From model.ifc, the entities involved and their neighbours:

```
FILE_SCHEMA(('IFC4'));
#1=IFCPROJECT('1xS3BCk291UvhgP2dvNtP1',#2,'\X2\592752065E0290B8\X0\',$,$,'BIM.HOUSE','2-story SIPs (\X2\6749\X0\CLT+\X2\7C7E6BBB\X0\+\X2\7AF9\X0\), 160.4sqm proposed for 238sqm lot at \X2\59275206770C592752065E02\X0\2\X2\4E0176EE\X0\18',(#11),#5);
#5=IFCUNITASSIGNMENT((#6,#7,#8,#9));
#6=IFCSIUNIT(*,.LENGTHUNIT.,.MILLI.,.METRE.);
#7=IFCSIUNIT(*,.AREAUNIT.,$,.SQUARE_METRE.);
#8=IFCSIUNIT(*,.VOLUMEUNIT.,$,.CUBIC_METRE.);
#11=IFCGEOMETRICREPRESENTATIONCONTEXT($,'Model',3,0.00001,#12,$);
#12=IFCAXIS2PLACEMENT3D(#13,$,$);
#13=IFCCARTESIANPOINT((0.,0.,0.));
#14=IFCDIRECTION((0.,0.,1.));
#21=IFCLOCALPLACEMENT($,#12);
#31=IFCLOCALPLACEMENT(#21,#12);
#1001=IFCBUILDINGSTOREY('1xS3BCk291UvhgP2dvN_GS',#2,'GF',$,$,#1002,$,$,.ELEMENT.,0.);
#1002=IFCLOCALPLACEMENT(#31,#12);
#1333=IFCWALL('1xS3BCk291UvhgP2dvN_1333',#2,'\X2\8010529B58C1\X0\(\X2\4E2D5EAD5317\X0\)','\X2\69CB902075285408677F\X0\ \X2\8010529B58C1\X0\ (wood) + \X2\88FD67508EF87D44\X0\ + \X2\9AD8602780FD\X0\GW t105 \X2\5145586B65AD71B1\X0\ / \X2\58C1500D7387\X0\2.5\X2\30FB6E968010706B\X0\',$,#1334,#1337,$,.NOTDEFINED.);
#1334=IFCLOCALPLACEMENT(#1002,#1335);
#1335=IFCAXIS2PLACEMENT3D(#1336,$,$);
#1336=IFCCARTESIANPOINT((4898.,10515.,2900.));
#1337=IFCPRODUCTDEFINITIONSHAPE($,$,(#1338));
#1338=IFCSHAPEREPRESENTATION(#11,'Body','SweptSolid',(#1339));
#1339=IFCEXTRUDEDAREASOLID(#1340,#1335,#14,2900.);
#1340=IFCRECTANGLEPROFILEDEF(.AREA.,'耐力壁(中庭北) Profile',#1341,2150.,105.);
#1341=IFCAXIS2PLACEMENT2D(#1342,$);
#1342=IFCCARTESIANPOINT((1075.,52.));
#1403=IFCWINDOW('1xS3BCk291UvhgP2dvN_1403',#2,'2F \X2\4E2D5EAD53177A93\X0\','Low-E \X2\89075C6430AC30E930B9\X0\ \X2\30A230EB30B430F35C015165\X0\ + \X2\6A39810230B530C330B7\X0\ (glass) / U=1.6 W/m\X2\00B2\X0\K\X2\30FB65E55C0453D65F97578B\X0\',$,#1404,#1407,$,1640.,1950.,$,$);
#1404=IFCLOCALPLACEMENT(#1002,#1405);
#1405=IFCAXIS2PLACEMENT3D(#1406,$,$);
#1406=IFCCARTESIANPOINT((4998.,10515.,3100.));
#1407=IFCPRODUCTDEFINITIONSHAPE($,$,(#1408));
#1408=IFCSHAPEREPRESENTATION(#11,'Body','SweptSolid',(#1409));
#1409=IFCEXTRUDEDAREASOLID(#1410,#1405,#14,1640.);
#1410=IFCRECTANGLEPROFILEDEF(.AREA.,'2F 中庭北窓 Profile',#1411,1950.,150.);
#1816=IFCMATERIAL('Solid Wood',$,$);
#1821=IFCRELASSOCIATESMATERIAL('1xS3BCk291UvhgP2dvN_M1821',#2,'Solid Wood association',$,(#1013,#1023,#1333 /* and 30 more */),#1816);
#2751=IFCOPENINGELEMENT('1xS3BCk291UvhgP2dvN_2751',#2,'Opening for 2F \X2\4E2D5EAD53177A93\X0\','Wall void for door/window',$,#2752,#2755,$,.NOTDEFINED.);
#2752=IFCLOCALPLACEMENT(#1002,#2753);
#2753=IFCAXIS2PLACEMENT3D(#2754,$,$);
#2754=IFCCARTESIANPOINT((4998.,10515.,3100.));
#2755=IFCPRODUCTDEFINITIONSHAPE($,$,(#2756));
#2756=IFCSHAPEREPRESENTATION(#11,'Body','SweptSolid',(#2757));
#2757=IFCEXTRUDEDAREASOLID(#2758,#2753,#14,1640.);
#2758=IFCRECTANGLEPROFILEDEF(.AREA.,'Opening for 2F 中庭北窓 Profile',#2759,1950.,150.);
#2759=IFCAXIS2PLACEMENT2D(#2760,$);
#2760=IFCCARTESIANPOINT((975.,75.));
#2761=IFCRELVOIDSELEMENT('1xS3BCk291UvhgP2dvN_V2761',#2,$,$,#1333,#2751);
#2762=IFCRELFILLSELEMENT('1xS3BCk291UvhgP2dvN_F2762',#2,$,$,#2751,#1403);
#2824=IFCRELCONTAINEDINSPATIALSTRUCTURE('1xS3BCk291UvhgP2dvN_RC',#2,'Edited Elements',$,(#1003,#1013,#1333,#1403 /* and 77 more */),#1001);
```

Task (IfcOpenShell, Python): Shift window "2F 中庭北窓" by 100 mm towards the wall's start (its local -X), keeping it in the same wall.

```python
import ifcopenshell
import ifcopenshell.api.geometry
import ifcopenshell.util.placement

model = ifcopenshell.open("model.ifc")

window = model.by_guid("1xS3BCk291UvhgP2dvN_1403")
opening = window.FillsVoids[0].RelatingOpeningElement
wall = opening.VoidsElements[0].RelatingBuildingElement

wall_matrix = ifcopenshell.util.placement.get_local_placement(wall.ObjectPlacement)
shift = wall_matrix[:3, 0] * -100.0
before = ifcopenshell.util.placement.get_local_placement(window.ObjectPlacement)[:3, 3].copy()

# The window is not placed relative to its opening, so move both.
for product in (opening, window):
    matrix = ifcopenshell.util.placement.get_local_placement(product.ObjectPlacement)
    matrix[:3, 3] += shift
    ifcopenshell.api.geometry.edit_object_placement(model, product=product, matrix=matrix, is_si=False)

after = ifcopenshell.util.placement.get_local_placement(window.ObjectPlacement)[:3, 3]
print("window moved by", (after - before).round(3) + 0.0)

model.write("model_rev.ifc")
```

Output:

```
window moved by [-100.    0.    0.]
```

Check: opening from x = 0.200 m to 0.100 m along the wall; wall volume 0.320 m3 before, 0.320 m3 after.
